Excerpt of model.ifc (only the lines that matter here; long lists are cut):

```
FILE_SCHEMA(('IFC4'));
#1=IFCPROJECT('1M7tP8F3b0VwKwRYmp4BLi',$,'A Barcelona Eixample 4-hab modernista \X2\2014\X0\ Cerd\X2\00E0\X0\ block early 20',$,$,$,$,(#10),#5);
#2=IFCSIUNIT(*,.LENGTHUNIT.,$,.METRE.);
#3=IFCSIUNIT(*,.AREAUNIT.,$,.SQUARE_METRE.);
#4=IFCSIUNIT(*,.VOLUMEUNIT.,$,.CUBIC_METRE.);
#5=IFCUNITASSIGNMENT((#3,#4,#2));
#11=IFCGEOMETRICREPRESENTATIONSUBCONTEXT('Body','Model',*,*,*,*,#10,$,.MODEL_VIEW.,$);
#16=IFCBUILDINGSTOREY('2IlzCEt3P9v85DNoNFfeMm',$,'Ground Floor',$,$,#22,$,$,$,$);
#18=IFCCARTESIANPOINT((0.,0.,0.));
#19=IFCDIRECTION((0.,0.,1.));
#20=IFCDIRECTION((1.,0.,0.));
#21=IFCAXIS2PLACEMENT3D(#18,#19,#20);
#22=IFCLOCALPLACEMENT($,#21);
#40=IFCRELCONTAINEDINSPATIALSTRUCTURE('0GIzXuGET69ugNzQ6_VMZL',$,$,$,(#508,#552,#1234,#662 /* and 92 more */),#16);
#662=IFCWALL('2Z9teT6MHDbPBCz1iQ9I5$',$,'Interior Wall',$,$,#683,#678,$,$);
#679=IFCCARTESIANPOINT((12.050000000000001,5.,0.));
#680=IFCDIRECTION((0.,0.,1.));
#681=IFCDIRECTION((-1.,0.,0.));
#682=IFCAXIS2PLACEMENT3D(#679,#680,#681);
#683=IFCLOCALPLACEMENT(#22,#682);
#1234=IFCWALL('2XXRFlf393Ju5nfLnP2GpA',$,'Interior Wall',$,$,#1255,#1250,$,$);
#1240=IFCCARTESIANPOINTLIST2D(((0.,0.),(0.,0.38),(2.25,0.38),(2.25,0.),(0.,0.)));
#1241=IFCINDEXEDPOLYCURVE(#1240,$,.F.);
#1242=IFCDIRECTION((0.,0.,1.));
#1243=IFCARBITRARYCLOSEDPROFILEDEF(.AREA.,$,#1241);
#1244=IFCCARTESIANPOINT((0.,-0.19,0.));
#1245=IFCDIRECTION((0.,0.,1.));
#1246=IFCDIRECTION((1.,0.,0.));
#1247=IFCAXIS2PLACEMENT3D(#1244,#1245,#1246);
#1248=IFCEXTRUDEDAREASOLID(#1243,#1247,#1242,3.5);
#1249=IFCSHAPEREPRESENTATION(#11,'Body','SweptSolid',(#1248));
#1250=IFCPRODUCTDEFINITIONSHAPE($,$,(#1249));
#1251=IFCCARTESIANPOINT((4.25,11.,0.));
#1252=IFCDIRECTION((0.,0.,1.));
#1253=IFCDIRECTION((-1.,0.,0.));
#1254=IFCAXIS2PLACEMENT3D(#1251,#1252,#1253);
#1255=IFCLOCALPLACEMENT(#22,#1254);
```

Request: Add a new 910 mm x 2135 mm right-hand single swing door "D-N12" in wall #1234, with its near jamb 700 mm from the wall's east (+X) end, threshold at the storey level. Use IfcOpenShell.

```python
import numpy as np
import ifcopenshell
import ifcopenshell.api.feature
import ifcopenshell.api.geometry
import ifcopenshell.api.root
import ifcopenshell.api.spatial
import ifcopenshell.geom
import ifcopenshell.util.element
import ifcopenshell.util.placement
import ifcopenshell.util.representation
import ifcopenshell.util.shape
import ifcopenshell.util.unit

model = ifcopenshell.open("model.ifc")
unit_scale = ifcopenshell.util.unit.calculate_unit_scale(model)
settings = ifcopenshell.geom.settings()


def volume(element):
    """Net volume in cubic metres, openings subtracted."""
    shape = ifcopenshell.geom.create_shape(settings, element)
    return ifcopenshell.util.shape.get_volume(shape.geometry)


wall = model.by_guid("2XXRFlf393Ju5nfLnP2GpA")
storey = ifcopenshell.util.element.get_container(wall, ifc_class="IfcBuildingStorey")
context = ifcopenshell.util.representation.get_context(model, "Model", "Body", "MODEL_VIEW")
before = volume(wall)

width, height, from_end, sill = 0.91, 2.135, 0.7, 0.0  # metres

# The wall runs along its own X axis, and the end named is its -X end.
wall_shape = ifcopenshell.geom.create_shape(settings, wall)
x, y, z = ifcopenshell.util.shape.get_vertices(wall_shape.geometry).T
start = x.min() + from_end
face, thickness = float(y.min()), float(y.max() - y.min())
wall_matrix = ifcopenshell.util.placement.get_local_placement(wall.ObjectPlacement)
level = ifcopenshell.util.placement.get_local_placement(storey.ObjectPlacement)[2, 3]


def in_wall(x, y):
    """Placement at x, y metres in the wall's axes, at sill height."""
    matrix = wall_matrix.copy()
    matrix[:, 3] = wall_matrix @ np.array([x / unit_scale, y / unit_scale, 0.0, 1.0])
    matrix[2, 3] = level + sill / unit_scale
    return matrix


# Opening: a box that overshoots both wall faces by 50 mm.
opening = ifcopenshell.api.root.create_entity(model, ifc_class="IfcOpeningElement", predefined_type="OPENING")
box = ifcopenshell.api.geometry.add_wall_representation(
    model, context=context, length=width, height=height, thickness=thickness + 0.1
)
ifcopenshell.api.geometry.assign_representation(model, product=opening, representation=box)
ifcopenshell.api.geometry.edit_object_placement(model, product=opening, matrix=in_wall(start, face - 0.05), is_si=False)
ifcopenshell.api.feature.add_feature(model, feature=opening, element=wall)

door = ifcopenshell.api.root.create_entity(model, ifc_class="IfcDoor", name="D-N12", predefined_type="DOOR")
door.OverallWidth, door.OverallHeight = width / unit_scale, height / unit_scale
door.OperationType = "SINGLE_SWING_RIGHT"
body = ifcopenshell.api.geometry.add_door_representation(
    model,
    context=context,
    overall_width=door.OverallWidth,
    overall_height=door.OverallHeight,
    operation_type="SINGLE_SWING_RIGHT",
    lining_properties={"LiningDepth": thickness / unit_scale, "ThresholdDepth": thickness / unit_scale},
)
ifcopenshell.api.geometry.assign_representation(model, product=door, representation=body)
ifcopenshell.api.spatial.assign_container(model, products=[door], relating_structure=storey)
ifcopenshell.api.feature.add_filling(model, opening=opening, element=door)

# The lining spans the wall, so the door starts at the wall face.
ifcopenshell.api.geometry.edit_object_placement(model, product=door, matrix=in_wall(start, face), is_si=False)

after = volume(wall)

print(f"wall volume {before:.3f} -> {after:.3f} m3")

model.write("model_edited.ifc")
```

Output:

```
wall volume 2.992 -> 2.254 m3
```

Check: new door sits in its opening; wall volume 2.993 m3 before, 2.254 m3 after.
